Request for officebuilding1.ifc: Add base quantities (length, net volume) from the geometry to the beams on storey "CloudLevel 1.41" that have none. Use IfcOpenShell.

First a look at what the model holds.

```python
import ifcopenshell
import ifcopenshell.util.element
import ifcopenshell.util.unit

model = ifcopenshell.open("officebuilding1.ifc")
print(model.schema)
for unit_type in ("LENGTHUNIT", "AREAUNIT", "VOLUMEUNIT"):
    print(unit_type, ifcopenshell.util.unit.calculate_unit_scale(model, unit_type))
storey = next(s for s in model.by_type("IfcBuildingStorey") if s.Name == "CloudLevel 1.41")
beams = [e for e in ifcopenshell.util.element.get_decomposition(storey) if e.is_a("IfcBeam")]
for e in sorted(beams, key=lambda e: e.id()):
    print(e.id(), e.is_a(), e.Name, list(ifcopenshell.util.element.get_psets(e, qtos_only=True)), sep=" | ")
```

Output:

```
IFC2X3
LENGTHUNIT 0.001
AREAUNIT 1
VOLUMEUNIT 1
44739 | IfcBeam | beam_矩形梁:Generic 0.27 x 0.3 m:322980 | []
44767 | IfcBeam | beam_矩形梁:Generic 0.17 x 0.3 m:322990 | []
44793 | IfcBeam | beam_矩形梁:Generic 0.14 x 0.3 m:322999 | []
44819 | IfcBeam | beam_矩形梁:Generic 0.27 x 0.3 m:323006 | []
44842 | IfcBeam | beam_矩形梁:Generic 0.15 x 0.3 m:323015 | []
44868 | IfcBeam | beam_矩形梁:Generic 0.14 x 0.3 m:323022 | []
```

```python
import ifcopenshell
import ifcopenshell.api.pset
import ifcopenshell.geom
import ifcopenshell.util.element
import ifcopenshell.util.shape
import ifcopenshell.util.unit

model = ifcopenshell.open("officebuilding1.ifc")
unit_scale = ifcopenshell.util.unit.calculate_unit_scale(model)
volume_scale = ifcopenshell.util.unit.calculate_unit_scale(model, "VOLUMEUNIT")
settings = ifcopenshell.geom.settings()

storey = next(s for s in model.by_type("IfcBuildingStorey") if s.Name == "CloudLevel 1.41")
beams = [e for e in ifcopenshell.util.element.get_decomposition(storey) if e.is_a("IfcBeam")]

for e in sorted(beams, key=lambda e: e.id()):
    if ifcopenshell.util.element.get_psets(e, qtos_only=True, should_inherit=False):
        continue
    # Geometry comes back in metres, in the element's own axes.
    shape = ifcopenshell.geom.create_shape(settings, e)
    values = {
        "Length": ifcopenshell.util.shape.get_max_xyz(shape.geometry) / unit_scale,
        "NetVolume": ifcopenshell.util.shape.get_volume(shape.geometry) / volume_scale,
    }
    qto = ifcopenshell.api.pset.add_qto(model, product=e, name="BaseQuantities")
    ifcopenshell.api.pset.edit_qto(model, qto=qto, properties=values)
    print(e.id(), {k: round(v, 3) for k, v in values.items()})

model.write("officebuilding1_rev.ifc")
```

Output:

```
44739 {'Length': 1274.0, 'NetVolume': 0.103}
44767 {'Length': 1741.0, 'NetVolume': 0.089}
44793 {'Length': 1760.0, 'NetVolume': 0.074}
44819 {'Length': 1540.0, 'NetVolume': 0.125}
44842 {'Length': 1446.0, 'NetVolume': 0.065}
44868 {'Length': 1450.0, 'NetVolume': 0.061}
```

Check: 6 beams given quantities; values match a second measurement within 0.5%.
